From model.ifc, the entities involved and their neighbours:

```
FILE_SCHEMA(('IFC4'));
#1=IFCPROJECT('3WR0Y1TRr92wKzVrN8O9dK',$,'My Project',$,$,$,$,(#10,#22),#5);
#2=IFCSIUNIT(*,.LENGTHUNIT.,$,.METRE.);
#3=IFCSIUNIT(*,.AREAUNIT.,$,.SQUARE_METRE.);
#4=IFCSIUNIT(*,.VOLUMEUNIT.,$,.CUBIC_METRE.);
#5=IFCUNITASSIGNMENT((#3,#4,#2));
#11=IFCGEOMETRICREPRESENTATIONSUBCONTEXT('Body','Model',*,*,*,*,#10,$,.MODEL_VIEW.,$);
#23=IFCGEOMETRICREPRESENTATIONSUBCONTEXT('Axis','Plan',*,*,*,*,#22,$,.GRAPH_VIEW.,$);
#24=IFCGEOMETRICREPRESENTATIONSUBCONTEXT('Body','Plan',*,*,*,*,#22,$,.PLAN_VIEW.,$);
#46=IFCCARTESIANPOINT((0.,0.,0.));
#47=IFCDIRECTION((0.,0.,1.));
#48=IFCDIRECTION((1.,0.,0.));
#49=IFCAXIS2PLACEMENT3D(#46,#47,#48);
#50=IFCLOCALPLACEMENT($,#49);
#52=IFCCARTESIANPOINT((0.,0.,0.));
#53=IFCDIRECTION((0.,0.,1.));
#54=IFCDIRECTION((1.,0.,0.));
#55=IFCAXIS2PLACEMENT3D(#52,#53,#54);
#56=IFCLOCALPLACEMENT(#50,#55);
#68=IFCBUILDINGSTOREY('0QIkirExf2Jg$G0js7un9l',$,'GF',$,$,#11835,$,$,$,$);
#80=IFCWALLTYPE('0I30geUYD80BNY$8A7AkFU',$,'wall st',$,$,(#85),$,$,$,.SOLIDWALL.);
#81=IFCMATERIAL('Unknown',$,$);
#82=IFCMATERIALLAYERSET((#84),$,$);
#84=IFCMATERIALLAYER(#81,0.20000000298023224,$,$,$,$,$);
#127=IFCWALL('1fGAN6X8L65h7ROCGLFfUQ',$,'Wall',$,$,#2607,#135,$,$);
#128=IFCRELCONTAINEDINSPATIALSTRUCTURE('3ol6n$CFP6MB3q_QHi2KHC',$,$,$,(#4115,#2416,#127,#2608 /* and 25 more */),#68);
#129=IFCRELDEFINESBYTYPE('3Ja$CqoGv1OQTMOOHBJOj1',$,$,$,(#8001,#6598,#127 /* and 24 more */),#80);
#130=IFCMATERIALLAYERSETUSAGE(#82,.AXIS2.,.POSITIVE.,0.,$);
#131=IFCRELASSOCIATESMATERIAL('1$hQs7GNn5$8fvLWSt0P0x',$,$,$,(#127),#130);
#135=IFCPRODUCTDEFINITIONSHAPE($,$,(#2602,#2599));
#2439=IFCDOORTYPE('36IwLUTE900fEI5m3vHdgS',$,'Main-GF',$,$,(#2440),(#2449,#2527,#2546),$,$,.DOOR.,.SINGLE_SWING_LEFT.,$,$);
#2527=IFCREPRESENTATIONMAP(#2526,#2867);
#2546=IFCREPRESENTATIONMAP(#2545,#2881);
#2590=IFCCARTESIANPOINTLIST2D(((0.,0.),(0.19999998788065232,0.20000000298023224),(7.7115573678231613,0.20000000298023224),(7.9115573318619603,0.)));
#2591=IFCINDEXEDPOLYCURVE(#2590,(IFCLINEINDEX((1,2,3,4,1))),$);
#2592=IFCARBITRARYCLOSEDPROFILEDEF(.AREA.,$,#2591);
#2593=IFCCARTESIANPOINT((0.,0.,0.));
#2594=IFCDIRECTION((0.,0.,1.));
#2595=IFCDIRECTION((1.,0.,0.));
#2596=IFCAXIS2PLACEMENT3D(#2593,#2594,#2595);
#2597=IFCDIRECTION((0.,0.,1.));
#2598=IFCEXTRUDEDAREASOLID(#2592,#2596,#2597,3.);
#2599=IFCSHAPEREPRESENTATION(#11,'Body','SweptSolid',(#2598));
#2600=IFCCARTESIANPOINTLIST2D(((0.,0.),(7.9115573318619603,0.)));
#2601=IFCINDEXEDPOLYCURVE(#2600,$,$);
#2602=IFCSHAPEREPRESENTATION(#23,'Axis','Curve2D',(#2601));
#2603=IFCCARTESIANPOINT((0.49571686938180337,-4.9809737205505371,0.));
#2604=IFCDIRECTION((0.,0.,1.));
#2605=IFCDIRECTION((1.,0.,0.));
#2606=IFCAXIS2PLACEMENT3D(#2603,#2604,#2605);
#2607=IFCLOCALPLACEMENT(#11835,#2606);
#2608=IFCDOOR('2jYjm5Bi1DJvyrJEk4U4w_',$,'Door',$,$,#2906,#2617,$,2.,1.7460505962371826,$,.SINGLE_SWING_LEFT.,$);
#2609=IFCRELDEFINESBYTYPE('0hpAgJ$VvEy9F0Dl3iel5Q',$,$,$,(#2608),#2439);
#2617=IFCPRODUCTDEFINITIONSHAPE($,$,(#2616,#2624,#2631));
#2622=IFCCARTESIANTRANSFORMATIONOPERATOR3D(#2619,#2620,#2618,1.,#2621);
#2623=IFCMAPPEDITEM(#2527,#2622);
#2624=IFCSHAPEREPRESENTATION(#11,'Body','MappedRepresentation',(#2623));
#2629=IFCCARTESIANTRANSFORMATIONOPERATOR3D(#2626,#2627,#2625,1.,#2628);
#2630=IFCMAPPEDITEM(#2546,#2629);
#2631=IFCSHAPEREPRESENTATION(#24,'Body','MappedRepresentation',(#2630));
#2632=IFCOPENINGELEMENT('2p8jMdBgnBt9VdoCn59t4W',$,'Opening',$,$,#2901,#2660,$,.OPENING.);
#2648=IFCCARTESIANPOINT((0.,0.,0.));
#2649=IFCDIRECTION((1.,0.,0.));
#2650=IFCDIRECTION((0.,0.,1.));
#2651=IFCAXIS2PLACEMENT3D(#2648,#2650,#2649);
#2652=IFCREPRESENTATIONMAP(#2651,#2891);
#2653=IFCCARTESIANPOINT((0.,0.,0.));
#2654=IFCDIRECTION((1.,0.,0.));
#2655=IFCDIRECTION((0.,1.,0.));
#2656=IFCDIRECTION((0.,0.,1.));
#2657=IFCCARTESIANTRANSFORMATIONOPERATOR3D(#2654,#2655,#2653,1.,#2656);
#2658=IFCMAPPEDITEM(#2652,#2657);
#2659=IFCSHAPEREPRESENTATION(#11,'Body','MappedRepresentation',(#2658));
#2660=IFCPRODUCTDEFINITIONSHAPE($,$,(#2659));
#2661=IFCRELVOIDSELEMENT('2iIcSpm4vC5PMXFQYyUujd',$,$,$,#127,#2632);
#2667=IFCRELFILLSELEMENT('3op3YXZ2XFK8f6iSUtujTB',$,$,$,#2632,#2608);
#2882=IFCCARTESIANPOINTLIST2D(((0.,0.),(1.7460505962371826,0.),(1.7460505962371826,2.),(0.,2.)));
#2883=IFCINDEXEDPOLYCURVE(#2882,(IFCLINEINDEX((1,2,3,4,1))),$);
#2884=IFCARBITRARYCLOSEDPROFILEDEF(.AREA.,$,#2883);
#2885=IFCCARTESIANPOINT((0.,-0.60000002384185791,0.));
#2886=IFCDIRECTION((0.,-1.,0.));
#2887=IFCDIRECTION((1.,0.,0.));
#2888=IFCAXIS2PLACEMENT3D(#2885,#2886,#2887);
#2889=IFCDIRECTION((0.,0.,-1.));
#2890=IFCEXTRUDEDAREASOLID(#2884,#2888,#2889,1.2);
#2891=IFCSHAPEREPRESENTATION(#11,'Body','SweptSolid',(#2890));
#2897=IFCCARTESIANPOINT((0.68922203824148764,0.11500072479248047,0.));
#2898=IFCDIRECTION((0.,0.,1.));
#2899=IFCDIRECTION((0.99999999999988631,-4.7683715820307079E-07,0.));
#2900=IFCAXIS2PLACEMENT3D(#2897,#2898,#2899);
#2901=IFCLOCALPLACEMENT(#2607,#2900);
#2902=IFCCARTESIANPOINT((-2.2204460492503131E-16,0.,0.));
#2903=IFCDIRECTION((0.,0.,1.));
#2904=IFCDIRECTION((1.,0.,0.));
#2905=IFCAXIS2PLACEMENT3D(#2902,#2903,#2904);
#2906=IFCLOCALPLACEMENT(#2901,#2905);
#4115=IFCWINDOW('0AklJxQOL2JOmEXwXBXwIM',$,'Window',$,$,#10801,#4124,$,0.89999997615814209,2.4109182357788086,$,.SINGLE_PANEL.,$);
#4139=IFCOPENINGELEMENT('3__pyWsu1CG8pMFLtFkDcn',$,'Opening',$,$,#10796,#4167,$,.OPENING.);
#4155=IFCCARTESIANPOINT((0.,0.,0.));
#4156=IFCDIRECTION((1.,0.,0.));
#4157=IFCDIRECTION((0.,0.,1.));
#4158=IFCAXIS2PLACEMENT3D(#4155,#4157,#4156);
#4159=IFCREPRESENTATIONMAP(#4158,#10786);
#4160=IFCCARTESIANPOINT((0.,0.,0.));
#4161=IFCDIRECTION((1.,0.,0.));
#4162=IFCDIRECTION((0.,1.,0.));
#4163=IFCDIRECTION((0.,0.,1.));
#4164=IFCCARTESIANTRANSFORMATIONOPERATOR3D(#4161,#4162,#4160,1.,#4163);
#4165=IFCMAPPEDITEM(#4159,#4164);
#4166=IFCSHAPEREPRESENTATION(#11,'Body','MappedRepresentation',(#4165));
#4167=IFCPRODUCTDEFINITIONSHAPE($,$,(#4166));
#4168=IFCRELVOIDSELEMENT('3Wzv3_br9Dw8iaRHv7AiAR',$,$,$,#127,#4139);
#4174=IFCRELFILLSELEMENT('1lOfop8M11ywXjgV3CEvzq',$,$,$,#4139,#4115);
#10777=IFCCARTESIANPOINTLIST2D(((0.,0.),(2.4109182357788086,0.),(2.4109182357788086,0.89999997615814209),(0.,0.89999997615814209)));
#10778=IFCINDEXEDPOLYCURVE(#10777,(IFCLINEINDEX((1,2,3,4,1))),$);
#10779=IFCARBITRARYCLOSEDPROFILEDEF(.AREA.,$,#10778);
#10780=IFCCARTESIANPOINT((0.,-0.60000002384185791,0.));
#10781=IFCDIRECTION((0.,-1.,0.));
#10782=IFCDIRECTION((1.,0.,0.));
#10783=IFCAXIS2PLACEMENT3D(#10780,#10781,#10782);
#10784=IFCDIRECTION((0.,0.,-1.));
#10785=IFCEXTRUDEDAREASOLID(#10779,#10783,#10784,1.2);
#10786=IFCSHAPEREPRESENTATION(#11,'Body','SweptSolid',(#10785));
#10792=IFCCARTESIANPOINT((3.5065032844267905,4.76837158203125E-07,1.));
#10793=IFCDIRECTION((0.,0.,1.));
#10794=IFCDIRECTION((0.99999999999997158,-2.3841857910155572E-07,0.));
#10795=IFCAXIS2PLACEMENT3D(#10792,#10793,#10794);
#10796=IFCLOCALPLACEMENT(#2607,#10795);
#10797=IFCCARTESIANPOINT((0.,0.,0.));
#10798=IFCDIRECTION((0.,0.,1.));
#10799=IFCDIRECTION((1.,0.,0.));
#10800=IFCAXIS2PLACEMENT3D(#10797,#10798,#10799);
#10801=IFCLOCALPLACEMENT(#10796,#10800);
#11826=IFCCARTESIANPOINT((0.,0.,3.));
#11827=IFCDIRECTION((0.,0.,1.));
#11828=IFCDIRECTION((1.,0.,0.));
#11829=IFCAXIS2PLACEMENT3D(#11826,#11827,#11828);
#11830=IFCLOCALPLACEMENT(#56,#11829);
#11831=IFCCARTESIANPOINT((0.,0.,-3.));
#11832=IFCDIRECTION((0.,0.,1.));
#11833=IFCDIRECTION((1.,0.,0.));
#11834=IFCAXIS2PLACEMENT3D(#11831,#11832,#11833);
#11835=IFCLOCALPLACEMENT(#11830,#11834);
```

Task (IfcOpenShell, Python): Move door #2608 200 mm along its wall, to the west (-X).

```python
import ifcopenshell
import ifcopenshell.api.geometry
import ifcopenshell.util.placement
import ifcopenshell.util.unit

model = ifcopenshell.open("model.ifc")
unit_scale = ifcopenshell.util.unit.calculate_unit_scale(model)

door = model.by_guid("2jYjm5Bi1DJvyrJEk4U4w_")
opening = door.FillsVoids[0].RelatingOpeningElement
wall = opening.VoidsElements[0].RelatingBuildingElement

wall_matrix = ifcopenshell.util.placement.get_local_placement(wall.ObjectPlacement)
shift = wall_matrix[:3, 0] * -0.2 / unit_scale
before = ifcopenshell.util.placement.get_local_placement(door.ObjectPlacement)[:3, 3].copy()

# The door is placed relative to its opening, so it follows when the opening moves.
matrix = ifcopenshell.util.placement.get_local_placement(opening.ObjectPlacement)
matrix[:3, 3] += shift
ifcopenshell.api.geometry.edit_object_placement(
    model, product=opening, matrix=matrix, is_si=False, should_transform_children=True
)

after = ifcopenshell.util.placement.get_local_placement(door.ObjectPlacement)[:3, 3]
print("door moved by", (after - before).round(3) + 0.0)

model.write("model_updated.ifc")
```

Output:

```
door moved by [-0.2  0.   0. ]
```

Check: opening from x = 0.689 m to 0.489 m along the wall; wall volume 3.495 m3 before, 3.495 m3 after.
